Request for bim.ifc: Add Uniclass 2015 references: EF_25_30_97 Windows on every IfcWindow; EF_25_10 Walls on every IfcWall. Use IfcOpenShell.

First a look at what the model holds.

```python
import ifcopenshell

model = ifcopenshell.open("bim.ifc")
print(model.schema)
print("classifications:", [c.Name for c in model.by_type("IfcClassification")])
for ifc_class in ("IfcDoor", "IfcRoof", "IfcStair", "IfcWall", "IfcWindow"):
    print(ifc_class, len(model.by_type(ifc_class)))
```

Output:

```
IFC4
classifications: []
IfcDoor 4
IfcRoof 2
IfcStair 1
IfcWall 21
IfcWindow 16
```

```python
import ifcopenshell
import ifcopenshell.api.classification

model = ifcopenshell.open("bim.ifc")

system = ifcopenshell.api.classification.add_classification(model, classification="Uniclass 2015")

codes = {
    "IfcWindow": ("EF_25_30_97", "Windows"),
    "IfcWall": ("EF_25_10", "Walls"),
}
for ifc_class, (code, name) in codes.items():
    products = model.by_type(ifc_class)
    ifcopenshell.api.classification.add_reference(
        model, products=products, classification=system, identification=code, name=name
    )
    print(code, len(products))

model.write("bim_v2.ifc")
```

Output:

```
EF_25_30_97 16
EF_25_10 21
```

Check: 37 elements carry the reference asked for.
